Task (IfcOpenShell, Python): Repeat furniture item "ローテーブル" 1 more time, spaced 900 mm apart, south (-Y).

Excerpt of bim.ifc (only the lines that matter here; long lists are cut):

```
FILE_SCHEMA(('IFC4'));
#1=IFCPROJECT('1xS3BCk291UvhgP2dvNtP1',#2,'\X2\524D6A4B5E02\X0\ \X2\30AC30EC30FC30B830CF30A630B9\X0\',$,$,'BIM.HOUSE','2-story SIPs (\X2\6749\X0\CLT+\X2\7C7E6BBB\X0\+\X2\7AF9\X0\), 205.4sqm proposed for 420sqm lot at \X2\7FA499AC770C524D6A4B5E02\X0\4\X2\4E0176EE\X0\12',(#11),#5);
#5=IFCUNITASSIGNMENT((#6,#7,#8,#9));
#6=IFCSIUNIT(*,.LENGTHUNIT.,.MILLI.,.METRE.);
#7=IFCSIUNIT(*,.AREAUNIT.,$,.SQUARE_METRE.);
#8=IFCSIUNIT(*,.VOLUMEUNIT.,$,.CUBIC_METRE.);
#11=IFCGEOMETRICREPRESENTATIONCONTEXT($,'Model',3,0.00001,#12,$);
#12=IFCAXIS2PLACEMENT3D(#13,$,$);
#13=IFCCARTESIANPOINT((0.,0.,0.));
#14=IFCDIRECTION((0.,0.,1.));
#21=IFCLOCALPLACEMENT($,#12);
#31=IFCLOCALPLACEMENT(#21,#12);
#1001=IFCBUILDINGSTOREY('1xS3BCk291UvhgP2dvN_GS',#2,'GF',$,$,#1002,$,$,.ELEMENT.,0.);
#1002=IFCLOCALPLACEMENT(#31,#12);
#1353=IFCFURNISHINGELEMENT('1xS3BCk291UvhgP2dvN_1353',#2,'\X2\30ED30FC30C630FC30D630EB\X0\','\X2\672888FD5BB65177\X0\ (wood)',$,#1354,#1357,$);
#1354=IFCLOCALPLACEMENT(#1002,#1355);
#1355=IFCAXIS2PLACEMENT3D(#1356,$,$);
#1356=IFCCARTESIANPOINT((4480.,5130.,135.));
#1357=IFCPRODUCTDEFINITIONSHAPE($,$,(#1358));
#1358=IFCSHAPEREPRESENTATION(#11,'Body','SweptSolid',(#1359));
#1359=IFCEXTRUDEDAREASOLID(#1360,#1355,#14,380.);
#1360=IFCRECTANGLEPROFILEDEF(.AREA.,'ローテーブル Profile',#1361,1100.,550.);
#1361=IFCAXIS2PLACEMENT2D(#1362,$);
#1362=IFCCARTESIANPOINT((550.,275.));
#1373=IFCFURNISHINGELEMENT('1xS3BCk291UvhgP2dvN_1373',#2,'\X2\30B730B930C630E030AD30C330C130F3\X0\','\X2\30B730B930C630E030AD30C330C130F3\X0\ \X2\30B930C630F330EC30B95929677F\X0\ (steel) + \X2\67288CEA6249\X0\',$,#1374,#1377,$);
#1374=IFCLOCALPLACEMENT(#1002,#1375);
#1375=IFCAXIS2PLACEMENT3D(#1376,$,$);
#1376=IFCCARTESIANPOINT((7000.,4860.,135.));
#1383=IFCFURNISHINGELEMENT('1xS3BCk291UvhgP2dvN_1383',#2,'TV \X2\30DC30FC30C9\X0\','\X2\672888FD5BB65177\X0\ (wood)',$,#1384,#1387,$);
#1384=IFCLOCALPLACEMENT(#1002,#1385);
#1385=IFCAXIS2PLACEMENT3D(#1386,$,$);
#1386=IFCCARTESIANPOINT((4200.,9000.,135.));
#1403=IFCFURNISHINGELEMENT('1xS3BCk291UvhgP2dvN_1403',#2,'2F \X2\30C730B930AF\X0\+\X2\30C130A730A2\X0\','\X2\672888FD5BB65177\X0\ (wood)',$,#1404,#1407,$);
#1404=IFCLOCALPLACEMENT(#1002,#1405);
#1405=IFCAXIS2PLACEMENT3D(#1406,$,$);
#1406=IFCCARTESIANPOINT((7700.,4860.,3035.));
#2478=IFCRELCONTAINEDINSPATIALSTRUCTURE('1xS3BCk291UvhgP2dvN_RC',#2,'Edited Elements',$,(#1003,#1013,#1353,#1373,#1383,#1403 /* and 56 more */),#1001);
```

```python
import numpy as np
import ifcopenshell
import ifcopenshell.api.geometry
import ifcopenshell.api.root
import ifcopenshell.util.element
import ifcopenshell.util.placement

model = ifcopenshell.open("bim.ifc")


def reuse_history(source, copy):
    """copy_class also copies each property set's owner history, people and application; keep the originals."""
    for rel in copy.IsDefinedBy:
        if rel.is_a("IfcRelDefinesByProperties") and (history := rel.RelatingPropertyDefinition.OwnerHistory):
            rel.RelatingPropertyDefinition.OwnerHistory = source.OwnerHistory
            ifcopenshell.util.element.remove_deep2(model, history)


source = model.by_guid("1xS3BCk291UvhgP2dvN_1353")
base = ifcopenshell.util.placement.get_local_placement(source.ObjectPlacement)
step = np.array([0.0, -1.0, 0.0]) * 900.0

for i in range(1, 2):
    copy = ifcopenshell.api.root.copy_class(model, product=source)
    copy.Representation = ifcopenshell.util.element.copy_deep(
        model, source.Representation, exclude=["IfcGeometricRepresentationContext", "IfcRepresentationMap"]
    )
    reuse_history(source, copy)
    matrix = base.copy()
    matrix[:3, 3] += i * step
    print("added at", matrix[:3, 3].round(3) + 0.0)
    ifcopenshell.api.geometry.edit_object_placement(model, product=copy, matrix=matrix, is_si=False)

model.write("bim_edited.ifc")
```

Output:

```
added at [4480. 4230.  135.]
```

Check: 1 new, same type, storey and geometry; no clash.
